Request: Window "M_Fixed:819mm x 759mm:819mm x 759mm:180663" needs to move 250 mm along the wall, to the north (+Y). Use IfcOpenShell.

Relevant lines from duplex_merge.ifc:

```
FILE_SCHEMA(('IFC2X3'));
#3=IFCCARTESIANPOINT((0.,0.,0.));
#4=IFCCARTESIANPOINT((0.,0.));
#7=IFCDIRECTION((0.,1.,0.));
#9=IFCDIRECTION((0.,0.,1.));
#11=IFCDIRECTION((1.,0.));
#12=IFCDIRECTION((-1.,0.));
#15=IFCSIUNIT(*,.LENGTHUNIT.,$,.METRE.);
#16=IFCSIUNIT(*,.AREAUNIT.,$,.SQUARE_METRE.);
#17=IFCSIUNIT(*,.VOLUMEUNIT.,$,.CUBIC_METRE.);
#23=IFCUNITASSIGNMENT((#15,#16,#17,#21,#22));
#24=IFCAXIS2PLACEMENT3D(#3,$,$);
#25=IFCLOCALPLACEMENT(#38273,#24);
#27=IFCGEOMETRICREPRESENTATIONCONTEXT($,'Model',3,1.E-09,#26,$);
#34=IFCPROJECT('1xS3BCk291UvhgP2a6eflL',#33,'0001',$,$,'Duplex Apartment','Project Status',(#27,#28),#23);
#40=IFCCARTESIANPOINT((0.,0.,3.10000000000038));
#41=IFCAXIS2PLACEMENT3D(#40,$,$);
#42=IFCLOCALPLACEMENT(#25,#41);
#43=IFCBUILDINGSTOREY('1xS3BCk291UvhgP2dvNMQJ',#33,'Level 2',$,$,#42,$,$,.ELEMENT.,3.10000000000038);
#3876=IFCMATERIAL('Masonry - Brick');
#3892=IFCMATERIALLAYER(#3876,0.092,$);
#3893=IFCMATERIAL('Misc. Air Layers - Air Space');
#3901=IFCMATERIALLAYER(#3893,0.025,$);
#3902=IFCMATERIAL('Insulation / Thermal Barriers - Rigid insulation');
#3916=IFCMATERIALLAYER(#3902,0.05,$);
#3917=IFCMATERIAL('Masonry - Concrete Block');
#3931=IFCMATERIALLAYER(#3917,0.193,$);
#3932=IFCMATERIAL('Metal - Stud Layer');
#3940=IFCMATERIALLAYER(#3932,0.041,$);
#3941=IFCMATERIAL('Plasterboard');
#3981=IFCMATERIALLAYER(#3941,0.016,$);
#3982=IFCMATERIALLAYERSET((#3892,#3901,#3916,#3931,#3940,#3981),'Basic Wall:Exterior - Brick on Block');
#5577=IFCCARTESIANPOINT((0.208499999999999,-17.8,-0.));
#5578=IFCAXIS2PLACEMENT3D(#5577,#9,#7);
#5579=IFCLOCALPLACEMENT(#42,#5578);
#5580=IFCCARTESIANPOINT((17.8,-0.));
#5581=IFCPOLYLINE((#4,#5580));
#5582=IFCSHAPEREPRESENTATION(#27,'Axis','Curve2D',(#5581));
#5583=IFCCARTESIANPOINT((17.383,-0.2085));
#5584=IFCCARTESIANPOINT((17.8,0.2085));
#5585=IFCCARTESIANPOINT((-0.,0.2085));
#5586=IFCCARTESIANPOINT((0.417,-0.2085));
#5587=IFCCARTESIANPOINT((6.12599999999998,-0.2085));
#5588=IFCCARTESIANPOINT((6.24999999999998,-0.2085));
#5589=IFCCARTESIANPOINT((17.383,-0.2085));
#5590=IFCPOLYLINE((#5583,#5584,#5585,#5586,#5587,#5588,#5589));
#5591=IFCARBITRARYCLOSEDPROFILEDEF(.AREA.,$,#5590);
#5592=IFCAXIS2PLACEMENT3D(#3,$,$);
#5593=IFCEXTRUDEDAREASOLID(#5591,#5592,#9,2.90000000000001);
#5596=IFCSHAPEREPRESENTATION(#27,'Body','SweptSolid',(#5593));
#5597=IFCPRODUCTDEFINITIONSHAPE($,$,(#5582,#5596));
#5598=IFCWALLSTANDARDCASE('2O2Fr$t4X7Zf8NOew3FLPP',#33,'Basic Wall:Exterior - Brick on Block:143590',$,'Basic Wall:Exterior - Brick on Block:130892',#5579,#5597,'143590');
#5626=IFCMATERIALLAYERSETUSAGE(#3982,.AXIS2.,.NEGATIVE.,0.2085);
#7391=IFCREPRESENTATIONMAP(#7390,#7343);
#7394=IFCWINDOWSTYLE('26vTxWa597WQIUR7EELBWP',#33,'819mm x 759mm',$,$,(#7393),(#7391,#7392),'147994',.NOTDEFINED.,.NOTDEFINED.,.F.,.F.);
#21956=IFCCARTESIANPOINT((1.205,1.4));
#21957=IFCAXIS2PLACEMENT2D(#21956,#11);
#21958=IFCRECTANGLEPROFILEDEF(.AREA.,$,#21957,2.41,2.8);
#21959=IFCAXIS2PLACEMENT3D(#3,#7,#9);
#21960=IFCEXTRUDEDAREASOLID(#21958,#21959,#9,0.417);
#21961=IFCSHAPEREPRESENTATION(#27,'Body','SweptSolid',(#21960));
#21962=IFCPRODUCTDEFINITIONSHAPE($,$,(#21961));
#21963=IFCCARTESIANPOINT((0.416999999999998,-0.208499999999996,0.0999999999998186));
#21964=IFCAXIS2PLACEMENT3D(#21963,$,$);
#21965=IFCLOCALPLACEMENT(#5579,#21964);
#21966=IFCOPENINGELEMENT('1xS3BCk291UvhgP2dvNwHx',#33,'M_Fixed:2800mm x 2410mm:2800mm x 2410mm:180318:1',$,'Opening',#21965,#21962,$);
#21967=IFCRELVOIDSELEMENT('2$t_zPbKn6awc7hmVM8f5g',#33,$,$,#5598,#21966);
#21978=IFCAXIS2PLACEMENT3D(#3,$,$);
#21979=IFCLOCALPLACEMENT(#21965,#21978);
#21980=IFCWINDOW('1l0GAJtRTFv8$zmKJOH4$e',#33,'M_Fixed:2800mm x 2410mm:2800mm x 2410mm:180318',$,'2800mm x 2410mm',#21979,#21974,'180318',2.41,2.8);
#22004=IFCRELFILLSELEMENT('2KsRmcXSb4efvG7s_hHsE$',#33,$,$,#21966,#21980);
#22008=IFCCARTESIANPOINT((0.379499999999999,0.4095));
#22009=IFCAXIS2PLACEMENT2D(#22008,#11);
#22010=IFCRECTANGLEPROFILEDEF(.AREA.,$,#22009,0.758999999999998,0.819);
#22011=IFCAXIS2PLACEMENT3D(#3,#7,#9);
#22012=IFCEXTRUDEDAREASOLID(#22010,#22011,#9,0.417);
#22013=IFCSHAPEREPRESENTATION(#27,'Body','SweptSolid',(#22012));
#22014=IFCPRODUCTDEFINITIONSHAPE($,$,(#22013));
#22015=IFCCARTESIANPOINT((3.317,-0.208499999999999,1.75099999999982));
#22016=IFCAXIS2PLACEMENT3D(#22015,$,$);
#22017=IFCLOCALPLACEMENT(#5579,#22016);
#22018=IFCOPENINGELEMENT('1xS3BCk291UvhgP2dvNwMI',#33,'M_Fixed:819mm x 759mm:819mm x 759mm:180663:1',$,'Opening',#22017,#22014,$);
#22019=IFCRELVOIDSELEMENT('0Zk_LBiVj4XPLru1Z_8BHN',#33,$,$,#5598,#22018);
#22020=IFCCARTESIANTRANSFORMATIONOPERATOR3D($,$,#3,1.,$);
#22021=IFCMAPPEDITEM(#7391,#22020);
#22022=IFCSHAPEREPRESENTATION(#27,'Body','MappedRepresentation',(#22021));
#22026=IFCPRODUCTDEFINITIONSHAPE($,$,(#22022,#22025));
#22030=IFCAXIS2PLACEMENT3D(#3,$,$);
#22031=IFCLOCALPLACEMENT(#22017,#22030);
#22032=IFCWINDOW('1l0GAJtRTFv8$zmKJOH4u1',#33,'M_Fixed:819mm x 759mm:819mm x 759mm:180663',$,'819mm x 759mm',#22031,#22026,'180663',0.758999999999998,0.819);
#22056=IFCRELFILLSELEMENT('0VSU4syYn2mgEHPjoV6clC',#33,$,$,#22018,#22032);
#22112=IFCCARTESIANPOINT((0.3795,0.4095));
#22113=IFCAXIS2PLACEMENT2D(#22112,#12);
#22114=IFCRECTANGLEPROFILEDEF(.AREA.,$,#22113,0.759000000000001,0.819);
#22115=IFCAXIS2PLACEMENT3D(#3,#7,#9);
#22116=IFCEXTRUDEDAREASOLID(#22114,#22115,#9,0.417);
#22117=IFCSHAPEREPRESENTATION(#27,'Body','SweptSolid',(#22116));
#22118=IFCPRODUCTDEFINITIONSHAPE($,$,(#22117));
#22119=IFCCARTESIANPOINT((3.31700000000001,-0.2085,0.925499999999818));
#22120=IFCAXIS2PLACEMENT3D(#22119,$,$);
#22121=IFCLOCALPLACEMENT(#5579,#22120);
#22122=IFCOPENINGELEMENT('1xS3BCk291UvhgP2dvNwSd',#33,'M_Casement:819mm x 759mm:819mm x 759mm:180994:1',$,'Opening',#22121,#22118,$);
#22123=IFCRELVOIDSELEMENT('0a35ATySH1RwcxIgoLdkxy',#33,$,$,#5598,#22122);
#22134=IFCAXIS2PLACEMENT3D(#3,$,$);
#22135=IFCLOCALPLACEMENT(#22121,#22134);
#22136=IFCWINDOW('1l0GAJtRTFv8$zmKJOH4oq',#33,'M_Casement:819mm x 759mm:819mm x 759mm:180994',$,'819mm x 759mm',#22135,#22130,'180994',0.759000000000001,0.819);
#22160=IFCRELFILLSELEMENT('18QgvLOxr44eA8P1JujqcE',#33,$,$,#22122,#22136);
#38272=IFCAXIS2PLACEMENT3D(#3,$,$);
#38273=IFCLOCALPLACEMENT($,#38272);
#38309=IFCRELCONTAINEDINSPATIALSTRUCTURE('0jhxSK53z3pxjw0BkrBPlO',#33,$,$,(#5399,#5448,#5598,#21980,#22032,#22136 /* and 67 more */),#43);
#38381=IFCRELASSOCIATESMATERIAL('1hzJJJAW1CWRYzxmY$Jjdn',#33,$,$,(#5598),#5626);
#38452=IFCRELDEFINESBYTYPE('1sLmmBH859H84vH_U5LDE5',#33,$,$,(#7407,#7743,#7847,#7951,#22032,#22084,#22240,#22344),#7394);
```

```python
import ifcopenshell
import ifcopenshell.api.geometry
import ifcopenshell.util.placement
import ifcopenshell.util.unit

model = ifcopenshell.open("duplex_merge.ifc")
unit_scale = ifcopenshell.util.unit.calculate_unit_scale(model)

window = model.by_guid("1l0GAJtRTFv8$zmKJOH4u1")
opening = window.FillsVoids[0].RelatingOpeningElement
wall = opening.VoidsElements[0].RelatingBuildingElement

wall_matrix = ifcopenshell.util.placement.get_local_placement(wall.ObjectPlacement)
shift = wall_matrix[:3, 0] * 0.25 / unit_scale
before = ifcopenshell.util.placement.get_local_placement(window.ObjectPlacement)[:3, 3].copy()

# The window is placed relative to its opening, so it follows when the opening moves.
matrix = ifcopenshell.util.placement.get_local_placement(opening.ObjectPlacement)
matrix[:3, 3] += shift
ifcopenshell.api.geometry.edit_object_placement(
    model, product=opening, matrix=matrix, is_si=False, should_transform_children=True
)

after = ifcopenshell.util.placement.get_local_placement(window.ObjectPlacement)[:3, 3]
print("window moved by", (after - before).round(3) + 0.0)

model.write("duplex_merge_v2.ifc")
```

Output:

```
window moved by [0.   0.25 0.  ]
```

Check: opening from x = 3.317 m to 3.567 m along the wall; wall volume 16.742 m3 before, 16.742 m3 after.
